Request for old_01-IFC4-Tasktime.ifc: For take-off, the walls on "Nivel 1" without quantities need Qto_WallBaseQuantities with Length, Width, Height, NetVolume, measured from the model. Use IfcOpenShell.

First a look at what the model holds.

```python
import ifcopenshell
import ifcopenshell.util.element
import ifcopenshell.util.unit

model = ifcopenshell.open("old_01-IFC4-Tasktime.ifc")
print(model.schema)
for unit_type in ("LENGTHUNIT", "AREAUNIT", "VOLUMEUNIT"):
    print(unit_type, ifcopenshell.util.unit.calculate_unit_scale(model, unit_type))
storey = next(s for s in model.by_type("IfcBuildingStorey") if s.Name == "Nivel 1")
walls = [e for e in ifcopenshell.util.element.get_decomposition(storey) if e.is_a("IfcWall")]
for e in sorted(walls, key=lambda e: e.id()):
    print(e.id(), e.is_a(), e.Name, list(ifcopenshell.util.element.get_psets(e, qtos_only=True)), sep=" | ")
```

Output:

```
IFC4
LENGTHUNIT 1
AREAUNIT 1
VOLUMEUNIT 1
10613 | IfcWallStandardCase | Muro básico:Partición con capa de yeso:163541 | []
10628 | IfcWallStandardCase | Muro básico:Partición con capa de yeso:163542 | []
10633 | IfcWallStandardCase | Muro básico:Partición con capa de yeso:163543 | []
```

```python
import ifcopenshell
import ifcopenshell.api.pset
import ifcopenshell.geom
import ifcopenshell.util.element
import ifcopenshell.util.shape
import ifcopenshell.util.unit

model = ifcopenshell.open("old_01-IFC4-Tasktime.ifc")
unit_scale = ifcopenshell.util.unit.calculate_unit_scale(model)
volume_scale = ifcopenshell.util.unit.calculate_unit_scale(model, "VOLUMEUNIT")
settings = ifcopenshell.geom.settings()

storey = next(s for s in model.by_type("IfcBuildingStorey") if s.Name == "Nivel 1")
walls = [e for e in ifcopenshell.util.element.get_decomposition(storey) if e.is_a("IfcWall")]

for e in sorted(walls, key=lambda e: e.id()):
    if ifcopenshell.util.element.get_psets(e, qtos_only=True, should_inherit=False):
        continue
    # Geometry comes back in metres, in the element's own axes.
    shape = ifcopenshell.geom.create_shape(settings, e)
    values = {
        "Length": ifcopenshell.util.shape.get_x(shape.geometry) / unit_scale,
        "Width": ifcopenshell.util.shape.get_y(shape.geometry) / unit_scale,
        "Height": ifcopenshell.util.shape.get_z(shape.geometry) / unit_scale,
        "NetVolume": ifcopenshell.util.shape.get_volume(shape.geometry) / volume_scale,
    }
    qto = ifcopenshell.api.pset.add_qto(model, product=e, name="Qto_WallBaseQuantities")
    ifcopenshell.api.pset.edit_qto(model, qto=qto, properties=values)
    print(e.id(), {k: round(v, 3) for k, v in values.items()})

model.write("old_01-IFC4-Tasktime_updated.ifc")
```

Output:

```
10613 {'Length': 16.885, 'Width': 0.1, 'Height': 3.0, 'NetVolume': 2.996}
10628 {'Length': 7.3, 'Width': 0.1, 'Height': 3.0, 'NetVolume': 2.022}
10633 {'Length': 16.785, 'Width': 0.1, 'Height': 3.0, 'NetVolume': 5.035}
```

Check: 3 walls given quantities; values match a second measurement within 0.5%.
